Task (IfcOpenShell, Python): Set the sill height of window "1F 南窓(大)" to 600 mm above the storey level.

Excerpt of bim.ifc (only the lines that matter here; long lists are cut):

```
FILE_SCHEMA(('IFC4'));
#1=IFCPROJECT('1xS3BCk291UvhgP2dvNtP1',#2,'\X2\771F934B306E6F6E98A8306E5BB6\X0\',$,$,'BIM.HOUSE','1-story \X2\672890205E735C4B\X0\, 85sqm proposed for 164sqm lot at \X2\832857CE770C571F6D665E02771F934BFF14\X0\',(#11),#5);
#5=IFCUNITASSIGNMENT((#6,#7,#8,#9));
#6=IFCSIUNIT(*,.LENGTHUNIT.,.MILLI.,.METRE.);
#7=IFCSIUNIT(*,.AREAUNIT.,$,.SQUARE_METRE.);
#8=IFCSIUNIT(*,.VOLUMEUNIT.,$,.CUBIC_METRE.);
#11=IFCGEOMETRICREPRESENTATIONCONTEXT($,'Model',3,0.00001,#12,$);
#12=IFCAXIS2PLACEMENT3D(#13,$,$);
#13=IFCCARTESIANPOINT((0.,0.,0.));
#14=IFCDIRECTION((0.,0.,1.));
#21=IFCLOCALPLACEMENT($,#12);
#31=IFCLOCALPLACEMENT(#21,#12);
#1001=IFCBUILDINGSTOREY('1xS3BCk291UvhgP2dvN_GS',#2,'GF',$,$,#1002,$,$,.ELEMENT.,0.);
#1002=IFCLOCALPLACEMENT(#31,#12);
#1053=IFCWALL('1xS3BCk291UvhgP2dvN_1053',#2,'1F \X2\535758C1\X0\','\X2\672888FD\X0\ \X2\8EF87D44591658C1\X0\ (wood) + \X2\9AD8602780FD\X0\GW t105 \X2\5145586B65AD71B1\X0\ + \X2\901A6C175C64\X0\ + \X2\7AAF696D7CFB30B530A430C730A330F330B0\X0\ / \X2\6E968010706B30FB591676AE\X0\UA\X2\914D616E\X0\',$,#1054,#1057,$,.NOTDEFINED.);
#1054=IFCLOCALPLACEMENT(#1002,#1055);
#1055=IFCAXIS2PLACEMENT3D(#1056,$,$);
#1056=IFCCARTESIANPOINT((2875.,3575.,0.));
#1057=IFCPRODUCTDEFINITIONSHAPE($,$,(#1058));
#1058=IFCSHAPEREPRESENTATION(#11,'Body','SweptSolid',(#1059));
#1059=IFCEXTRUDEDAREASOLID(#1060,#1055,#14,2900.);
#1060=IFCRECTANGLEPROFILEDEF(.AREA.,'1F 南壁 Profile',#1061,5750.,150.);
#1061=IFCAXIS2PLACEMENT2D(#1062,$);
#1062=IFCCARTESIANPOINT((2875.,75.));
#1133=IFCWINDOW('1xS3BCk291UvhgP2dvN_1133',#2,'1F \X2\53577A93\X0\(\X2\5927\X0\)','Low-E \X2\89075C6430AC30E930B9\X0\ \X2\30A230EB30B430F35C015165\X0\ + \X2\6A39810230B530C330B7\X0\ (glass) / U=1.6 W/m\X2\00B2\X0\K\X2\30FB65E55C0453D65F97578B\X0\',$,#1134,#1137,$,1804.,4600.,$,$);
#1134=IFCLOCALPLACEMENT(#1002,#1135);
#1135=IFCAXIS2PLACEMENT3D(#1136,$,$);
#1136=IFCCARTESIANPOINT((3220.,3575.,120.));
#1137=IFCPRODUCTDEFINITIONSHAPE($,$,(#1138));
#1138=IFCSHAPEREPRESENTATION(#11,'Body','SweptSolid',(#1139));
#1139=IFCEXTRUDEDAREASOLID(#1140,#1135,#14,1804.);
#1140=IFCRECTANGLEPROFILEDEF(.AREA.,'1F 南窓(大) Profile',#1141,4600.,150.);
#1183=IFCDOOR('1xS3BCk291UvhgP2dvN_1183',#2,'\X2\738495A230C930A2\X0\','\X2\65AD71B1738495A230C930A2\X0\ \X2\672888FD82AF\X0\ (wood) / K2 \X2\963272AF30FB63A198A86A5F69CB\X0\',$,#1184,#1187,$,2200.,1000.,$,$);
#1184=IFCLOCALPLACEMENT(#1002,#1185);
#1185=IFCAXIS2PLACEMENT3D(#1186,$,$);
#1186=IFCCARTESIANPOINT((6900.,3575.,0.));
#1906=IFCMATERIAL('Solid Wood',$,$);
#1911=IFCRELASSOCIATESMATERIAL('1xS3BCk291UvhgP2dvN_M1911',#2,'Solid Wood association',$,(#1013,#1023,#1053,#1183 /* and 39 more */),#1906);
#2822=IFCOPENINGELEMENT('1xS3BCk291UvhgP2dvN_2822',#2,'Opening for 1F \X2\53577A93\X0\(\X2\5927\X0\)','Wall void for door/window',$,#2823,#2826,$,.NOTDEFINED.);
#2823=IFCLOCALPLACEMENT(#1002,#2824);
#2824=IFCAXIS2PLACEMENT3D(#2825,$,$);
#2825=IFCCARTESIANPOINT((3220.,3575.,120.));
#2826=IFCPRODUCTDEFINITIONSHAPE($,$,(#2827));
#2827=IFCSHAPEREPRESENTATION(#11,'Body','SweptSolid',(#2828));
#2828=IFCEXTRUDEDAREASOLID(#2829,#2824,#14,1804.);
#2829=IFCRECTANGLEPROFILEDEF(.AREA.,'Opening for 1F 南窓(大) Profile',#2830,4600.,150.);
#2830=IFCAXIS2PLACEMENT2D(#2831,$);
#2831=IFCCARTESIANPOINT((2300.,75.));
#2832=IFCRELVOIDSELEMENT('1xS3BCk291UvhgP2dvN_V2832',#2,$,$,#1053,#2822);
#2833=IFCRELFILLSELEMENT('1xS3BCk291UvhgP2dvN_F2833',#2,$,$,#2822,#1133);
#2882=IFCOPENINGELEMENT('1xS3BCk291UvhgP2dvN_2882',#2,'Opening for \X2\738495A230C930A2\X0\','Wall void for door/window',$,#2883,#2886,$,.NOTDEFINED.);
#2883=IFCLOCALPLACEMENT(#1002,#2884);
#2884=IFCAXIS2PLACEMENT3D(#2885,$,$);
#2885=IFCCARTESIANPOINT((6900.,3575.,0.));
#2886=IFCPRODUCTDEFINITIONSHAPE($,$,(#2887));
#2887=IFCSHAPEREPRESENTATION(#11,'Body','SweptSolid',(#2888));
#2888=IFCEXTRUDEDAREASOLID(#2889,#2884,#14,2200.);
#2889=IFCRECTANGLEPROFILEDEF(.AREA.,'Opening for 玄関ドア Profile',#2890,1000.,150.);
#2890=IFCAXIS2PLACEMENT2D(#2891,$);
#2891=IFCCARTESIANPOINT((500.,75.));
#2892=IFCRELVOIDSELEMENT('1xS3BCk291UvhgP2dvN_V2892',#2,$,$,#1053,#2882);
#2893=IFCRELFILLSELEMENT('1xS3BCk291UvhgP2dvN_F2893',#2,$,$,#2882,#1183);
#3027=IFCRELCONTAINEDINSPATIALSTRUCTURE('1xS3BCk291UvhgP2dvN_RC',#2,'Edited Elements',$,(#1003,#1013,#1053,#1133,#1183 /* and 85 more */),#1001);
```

```python
import numpy as np
import ifcopenshell
import ifcopenshell.api.geometry
import ifcopenshell.geom
import ifcopenshell.util.element
import ifcopenshell.util.placement
import ifcopenshell.util.shape
import ifcopenshell.util.unit

model = ifcopenshell.open("bim.ifc")
unit_scale = ifcopenshell.util.unit.calculate_unit_scale(model)

window = model.by_guid("1xS3BCk291UvhgP2dvN_1133")
opening = window.FillsVoids[0].RelatingOpeningElement
storey = ifcopenshell.util.element.get_container(window, ifc_class="IfcBuildingStorey")
level = ifcopenshell.util.placement.get_local_placement(storey.ObjectPlacement)[2, 3]

# The opening's origin need not be at the sill, so measure its lowest point.
shape = ifcopenshell.geom.create_shape(ifcopenshell.geom.settings(), opening)
bottom = ifcopenshell.util.shape.get_shape_bottom_elevation(shape, shape.geometry) / unit_scale
dz = level + 0.6 / unit_scale - bottom

shift = np.array([0.0, 0.0, dz])
# The window is not placed relative to its opening, so move both.
for product in (opening, window):
    matrix = ifcopenshell.util.placement.get_local_placement(product.ObjectPlacement)
    matrix[:3, 3] += shift
    ifcopenshell.api.geometry.edit_object_placement(model, product=product, matrix=matrix, is_si=False)

print(f"moved by {dz * unit_scale:+.3f} m")

model.write("bim-out.ifc")
```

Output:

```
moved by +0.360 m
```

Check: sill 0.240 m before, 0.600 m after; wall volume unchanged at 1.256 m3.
